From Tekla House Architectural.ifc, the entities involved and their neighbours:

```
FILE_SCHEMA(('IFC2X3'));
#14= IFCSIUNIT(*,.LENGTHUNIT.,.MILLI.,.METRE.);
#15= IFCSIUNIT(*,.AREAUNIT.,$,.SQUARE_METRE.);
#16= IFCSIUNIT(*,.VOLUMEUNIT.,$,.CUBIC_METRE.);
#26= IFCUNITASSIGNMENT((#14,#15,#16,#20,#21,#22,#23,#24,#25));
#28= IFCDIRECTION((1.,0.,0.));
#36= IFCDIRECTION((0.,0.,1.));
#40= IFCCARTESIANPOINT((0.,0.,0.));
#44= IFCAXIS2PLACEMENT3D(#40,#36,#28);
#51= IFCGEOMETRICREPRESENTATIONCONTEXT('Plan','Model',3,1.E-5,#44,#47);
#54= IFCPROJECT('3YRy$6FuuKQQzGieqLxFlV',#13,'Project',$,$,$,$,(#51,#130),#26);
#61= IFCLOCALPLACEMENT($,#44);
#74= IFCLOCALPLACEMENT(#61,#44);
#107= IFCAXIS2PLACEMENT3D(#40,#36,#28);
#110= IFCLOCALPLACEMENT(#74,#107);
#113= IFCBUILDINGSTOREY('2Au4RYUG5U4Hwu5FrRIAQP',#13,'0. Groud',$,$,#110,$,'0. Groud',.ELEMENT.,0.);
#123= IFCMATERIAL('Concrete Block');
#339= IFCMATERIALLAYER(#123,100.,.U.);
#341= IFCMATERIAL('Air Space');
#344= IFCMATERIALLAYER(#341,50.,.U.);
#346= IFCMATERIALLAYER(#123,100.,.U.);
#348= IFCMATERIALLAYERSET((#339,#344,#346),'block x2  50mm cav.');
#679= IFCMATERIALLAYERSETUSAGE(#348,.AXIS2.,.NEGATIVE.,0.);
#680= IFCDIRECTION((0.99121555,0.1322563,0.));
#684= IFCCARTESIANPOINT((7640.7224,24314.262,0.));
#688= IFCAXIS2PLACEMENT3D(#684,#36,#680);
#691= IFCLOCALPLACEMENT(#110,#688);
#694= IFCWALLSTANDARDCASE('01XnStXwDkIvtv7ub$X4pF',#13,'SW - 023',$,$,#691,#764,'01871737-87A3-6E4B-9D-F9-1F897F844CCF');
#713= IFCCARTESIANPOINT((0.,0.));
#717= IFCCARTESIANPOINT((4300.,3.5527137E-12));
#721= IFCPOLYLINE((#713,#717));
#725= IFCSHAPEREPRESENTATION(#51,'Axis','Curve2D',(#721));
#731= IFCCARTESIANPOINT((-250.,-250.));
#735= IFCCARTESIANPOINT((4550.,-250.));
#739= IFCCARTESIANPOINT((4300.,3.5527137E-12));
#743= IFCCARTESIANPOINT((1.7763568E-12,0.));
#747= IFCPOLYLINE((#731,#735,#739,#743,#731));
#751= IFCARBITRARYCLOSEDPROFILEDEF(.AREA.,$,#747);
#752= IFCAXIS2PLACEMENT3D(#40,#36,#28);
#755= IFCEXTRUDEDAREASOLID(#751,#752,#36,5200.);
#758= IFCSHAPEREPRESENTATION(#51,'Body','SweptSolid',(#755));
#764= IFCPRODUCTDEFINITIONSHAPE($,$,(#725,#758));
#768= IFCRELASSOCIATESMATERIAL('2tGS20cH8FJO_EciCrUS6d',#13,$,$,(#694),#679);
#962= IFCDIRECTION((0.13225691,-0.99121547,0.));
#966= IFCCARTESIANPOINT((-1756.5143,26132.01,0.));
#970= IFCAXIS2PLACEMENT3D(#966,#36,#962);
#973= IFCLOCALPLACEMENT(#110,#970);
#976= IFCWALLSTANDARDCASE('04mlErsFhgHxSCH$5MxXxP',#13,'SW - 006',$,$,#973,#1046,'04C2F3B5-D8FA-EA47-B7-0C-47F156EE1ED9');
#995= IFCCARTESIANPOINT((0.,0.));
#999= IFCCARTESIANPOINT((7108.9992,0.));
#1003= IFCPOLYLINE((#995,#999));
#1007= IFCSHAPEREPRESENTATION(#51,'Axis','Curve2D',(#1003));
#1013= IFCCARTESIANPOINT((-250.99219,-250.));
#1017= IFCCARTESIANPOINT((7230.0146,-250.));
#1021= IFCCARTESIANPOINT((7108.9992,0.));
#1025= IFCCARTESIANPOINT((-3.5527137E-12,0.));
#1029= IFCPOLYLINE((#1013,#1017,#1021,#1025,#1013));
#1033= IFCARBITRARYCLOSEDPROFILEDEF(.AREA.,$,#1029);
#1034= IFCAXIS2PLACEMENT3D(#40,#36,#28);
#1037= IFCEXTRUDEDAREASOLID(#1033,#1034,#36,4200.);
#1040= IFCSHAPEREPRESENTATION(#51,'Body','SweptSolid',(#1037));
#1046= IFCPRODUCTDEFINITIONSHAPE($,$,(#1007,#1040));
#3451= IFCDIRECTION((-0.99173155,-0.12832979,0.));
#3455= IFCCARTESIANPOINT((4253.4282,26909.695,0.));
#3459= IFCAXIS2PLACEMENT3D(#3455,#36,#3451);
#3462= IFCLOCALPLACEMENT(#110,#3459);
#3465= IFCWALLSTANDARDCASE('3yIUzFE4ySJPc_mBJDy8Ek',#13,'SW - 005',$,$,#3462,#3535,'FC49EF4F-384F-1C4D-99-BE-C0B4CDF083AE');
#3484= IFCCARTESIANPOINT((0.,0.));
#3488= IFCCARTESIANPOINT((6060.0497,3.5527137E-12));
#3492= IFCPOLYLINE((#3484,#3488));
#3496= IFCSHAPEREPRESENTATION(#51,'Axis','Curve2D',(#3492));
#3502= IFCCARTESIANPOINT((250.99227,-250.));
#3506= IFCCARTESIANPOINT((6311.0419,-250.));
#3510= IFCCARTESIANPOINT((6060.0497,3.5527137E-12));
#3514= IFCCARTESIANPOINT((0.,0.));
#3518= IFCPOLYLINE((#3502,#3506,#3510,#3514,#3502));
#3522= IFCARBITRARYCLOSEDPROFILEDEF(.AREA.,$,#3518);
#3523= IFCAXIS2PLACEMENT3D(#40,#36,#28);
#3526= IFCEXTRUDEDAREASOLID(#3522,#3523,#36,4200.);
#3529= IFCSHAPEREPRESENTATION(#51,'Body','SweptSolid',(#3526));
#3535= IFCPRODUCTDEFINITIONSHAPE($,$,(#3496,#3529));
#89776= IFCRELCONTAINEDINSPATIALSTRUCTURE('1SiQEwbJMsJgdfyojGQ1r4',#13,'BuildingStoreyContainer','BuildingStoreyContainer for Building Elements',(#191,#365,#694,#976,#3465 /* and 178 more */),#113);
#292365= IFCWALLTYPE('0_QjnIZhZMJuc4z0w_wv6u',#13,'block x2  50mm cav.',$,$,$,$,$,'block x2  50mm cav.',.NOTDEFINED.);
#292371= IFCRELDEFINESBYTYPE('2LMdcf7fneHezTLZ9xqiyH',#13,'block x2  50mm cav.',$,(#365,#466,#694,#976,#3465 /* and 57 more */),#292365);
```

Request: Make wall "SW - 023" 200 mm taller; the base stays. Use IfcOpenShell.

```python
import ifcopenshell
import ifcopenshell.geom
import ifcopenshell.util.shape
import ifcopenshell.util.unit

model = ifcopenshell.open("Tekla House Architectural.ifc")
unit_scale = ifcopenshell.util.unit.calculate_unit_scale(model)
settings = ifcopenshell.geom.settings()


def volume(element):
    """Net volume in cubic metres, openings subtracted."""
    shape = ifcopenshell.geom.create_shape(settings, element)
    return ifcopenshell.util.shape.get_volume(shape.geometry)


wall = model.by_guid("01XnStXwDkIvtv7ub$X4pF")
before = volume(wall)

body = next(r for r in wall.Representation.Representations if r.RepresentationIdentifier == "Body")
solid = body.Items[0]
old_height = solid.Depth
solid.Depth += 0.2 / unit_scale
after = volume(wall)

print(f"height {old_height:g} -> {solid.Depth:g}, volume {before:.3f} -> {after:.3f} m3")

model.write("Tekla House Architectural_edited.ifc")
```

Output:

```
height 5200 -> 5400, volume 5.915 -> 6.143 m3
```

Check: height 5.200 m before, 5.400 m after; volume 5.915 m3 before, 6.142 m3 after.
